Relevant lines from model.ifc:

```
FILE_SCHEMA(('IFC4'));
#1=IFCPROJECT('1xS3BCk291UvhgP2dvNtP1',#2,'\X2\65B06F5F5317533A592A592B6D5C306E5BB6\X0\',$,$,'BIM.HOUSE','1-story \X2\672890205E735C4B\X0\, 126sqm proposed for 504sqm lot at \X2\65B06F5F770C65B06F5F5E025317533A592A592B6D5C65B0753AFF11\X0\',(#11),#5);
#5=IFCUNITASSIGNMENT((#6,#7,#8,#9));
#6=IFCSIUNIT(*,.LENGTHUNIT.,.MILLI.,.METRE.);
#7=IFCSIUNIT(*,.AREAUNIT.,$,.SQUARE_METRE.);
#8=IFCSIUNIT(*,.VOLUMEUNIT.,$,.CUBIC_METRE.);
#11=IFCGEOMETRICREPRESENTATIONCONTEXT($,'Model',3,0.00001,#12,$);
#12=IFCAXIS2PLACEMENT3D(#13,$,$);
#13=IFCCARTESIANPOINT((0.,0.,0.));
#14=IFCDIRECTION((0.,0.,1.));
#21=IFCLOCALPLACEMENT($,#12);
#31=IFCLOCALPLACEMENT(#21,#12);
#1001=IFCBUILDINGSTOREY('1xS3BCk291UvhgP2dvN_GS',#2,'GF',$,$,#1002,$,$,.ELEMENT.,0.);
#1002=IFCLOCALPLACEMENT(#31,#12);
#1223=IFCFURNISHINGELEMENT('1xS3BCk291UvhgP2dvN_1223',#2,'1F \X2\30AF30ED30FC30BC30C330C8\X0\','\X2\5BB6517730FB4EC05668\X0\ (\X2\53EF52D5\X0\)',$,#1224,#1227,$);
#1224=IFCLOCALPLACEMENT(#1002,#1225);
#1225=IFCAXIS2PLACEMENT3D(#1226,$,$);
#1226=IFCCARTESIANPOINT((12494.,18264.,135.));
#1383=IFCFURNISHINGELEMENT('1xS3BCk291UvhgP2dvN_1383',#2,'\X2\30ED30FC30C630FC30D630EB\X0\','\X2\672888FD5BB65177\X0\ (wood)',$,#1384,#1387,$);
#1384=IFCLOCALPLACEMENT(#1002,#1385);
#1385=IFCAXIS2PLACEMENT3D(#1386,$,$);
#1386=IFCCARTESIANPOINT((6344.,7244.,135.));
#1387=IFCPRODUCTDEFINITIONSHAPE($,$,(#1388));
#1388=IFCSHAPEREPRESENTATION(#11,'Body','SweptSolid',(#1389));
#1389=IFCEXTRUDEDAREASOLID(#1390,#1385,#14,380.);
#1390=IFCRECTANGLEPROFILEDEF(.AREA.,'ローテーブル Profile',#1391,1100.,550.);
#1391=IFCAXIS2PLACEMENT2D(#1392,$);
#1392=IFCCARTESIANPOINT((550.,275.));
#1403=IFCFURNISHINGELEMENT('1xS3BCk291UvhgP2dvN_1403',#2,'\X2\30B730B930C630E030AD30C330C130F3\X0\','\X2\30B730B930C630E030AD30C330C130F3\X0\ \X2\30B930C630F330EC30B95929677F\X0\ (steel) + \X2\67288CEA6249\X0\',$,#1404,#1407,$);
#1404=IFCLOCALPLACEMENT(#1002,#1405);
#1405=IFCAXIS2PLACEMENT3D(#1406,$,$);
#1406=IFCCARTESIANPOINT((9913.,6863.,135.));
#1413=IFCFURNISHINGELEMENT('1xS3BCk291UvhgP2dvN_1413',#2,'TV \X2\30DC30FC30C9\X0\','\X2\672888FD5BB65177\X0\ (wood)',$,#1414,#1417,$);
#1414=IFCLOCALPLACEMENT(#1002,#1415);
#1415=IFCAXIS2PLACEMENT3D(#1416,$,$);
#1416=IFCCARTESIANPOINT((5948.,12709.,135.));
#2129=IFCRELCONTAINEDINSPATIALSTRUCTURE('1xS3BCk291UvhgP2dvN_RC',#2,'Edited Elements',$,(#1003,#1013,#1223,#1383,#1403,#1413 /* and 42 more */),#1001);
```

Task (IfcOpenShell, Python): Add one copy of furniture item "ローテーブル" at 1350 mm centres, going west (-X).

```python
import numpy as np
import ifcopenshell
import ifcopenshell.api.geometry
import ifcopenshell.api.root
import ifcopenshell.util.element
import ifcopenshell.util.placement
import ifcopenshell.util.unit

model = ifcopenshell.open("model.ifc")
unit_scale = ifcopenshell.util.unit.calculate_unit_scale(model)


def reuse_history(source, copy):
    """copy_class also copies each property set's owner history, people and application; keep the originals."""
    for rel in copy.IsDefinedBy:
        if rel.is_a("IfcRelDefinesByProperties") and (history := rel.RelatingPropertyDefinition.OwnerHistory):
            rel.RelatingPropertyDefinition.OwnerHistory = source.OwnerHistory
            ifcopenshell.util.element.remove_deep2(model, history)


source = model.by_guid("1xS3BCk291UvhgP2dvN_1383")
base = ifcopenshell.util.placement.get_local_placement(source.ObjectPlacement)
step = np.array([-1.0, 0.0, 0.0]) * 1.35 / unit_scale

for i in range(1, 2):
    copy = ifcopenshell.api.root.copy_class(model, product=source)
    copy.Representation = ifcopenshell.util.element.copy_deep(
        model, source.Representation, exclude=["IfcGeometricRepresentationContext", "IfcRepresentationMap"]
    )
    reuse_history(source, copy)
    matrix = base.copy()
    matrix[:3, 3] += i * step
    print("added at", matrix[:3, 3].round(3) + 0.0)
    ifcopenshell.api.geometry.edit_object_placement(model, product=copy, matrix=matrix, is_si=False)

model.write("model_v2.ifc")
```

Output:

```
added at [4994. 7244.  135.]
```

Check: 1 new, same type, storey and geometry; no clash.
